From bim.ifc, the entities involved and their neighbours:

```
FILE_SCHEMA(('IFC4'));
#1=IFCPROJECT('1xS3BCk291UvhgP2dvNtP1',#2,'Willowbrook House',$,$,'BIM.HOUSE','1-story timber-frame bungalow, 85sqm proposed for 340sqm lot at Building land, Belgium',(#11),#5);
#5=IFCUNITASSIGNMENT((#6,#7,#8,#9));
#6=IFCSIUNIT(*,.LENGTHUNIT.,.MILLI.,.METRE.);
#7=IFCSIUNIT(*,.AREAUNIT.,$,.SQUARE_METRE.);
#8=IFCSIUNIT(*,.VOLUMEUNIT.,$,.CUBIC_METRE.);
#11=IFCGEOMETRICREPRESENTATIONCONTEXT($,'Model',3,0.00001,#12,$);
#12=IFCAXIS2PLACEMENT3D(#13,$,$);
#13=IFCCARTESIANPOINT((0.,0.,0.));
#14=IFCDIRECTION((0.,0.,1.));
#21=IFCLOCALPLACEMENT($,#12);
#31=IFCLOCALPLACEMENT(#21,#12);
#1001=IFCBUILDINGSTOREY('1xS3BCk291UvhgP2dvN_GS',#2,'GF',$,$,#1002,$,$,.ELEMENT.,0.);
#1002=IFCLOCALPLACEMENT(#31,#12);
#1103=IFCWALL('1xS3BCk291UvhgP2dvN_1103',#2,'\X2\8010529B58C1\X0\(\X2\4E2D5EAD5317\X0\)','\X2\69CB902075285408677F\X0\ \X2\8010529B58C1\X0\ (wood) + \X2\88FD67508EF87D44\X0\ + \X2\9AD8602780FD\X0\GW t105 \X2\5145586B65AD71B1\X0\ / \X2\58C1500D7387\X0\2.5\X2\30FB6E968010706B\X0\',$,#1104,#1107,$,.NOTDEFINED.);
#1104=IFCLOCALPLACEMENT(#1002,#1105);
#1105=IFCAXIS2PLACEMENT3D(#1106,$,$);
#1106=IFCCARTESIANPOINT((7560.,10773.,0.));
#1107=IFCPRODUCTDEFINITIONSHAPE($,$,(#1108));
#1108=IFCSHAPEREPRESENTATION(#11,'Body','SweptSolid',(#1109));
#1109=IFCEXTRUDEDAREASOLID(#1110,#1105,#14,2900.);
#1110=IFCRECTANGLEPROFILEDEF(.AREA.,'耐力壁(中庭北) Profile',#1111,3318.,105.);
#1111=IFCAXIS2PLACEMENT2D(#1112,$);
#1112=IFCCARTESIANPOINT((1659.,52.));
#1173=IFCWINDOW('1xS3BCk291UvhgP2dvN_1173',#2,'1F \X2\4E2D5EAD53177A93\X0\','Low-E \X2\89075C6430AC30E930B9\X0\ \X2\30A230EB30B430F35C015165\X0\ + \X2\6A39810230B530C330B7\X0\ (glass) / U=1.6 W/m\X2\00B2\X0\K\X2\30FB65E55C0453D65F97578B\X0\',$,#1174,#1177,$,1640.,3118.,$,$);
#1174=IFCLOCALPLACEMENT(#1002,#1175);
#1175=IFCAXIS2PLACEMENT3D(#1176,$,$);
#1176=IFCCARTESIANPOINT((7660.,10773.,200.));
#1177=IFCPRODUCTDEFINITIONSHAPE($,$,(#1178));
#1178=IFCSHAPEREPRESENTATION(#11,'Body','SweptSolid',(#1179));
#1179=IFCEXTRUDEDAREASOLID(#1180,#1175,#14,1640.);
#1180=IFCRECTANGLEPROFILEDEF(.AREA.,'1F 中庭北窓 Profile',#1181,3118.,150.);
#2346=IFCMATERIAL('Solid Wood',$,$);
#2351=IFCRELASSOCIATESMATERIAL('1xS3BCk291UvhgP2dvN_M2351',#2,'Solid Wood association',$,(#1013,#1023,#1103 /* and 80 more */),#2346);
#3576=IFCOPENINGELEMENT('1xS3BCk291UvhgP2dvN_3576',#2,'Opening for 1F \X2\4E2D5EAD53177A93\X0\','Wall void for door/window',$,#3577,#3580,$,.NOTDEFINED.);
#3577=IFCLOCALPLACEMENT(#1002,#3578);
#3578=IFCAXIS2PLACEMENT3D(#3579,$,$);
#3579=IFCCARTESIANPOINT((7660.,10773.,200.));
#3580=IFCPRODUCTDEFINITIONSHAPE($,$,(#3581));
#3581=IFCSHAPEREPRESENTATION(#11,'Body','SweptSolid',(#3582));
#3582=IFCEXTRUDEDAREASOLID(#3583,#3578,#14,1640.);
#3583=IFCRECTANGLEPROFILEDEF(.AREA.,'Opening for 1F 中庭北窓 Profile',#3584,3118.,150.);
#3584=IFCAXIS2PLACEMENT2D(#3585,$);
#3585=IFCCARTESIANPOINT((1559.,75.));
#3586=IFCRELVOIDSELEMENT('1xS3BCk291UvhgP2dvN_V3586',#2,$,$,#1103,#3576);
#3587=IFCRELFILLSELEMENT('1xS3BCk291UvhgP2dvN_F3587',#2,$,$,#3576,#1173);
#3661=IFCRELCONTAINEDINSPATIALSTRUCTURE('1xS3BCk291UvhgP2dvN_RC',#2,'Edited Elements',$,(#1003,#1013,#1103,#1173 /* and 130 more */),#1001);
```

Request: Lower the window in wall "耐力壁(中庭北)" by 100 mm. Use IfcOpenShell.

```python
import numpy as np
import ifcopenshell
import ifcopenshell.api.geometry
import ifcopenshell.util.placement
import ifcopenshell.util.unit

model = ifcopenshell.open("bim.ifc")
unit_scale = ifcopenshell.util.unit.calculate_unit_scale(model)

window = model.by_guid("1xS3BCk291UvhgP2dvN_1173")
opening = window.FillsVoids[0].RelatingOpeningElement
dz = -0.1 / unit_scale

shift = np.array([0.0, 0.0, dz])
# The window is not placed relative to its opening, so move both.
for product in (opening, window):
    matrix = ifcopenshell.util.placement.get_local_placement(product.ObjectPlacement)
    matrix[:3, 3] += shift
    ifcopenshell.api.geometry.edit_object_placement(model, product=product, matrix=matrix, is_si=False)

print(f"moved by {dz * unit_scale:+.3f} m")

model.write("bim-out.ifc")
```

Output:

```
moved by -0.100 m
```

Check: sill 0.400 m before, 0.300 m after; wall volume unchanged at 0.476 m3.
